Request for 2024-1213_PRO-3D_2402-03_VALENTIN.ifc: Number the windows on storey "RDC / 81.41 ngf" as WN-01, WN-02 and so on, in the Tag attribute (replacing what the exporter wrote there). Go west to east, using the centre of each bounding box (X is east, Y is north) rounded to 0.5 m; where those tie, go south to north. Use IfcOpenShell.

First a look at what the model holds.

```python
import ifcopenshell
import ifcopenshell.util.element
import ifcopenshell.util.placement

model = ifcopenshell.open("2024-1213_PRO-3D_2402-03_VALENTIN.ifc")
print(model.schema)
storey = next(s for s in model.by_type("IfcBuildingStorey") if s.Name == "RDC / 81.41 ngf")
windows = [e for e in ifcopenshell.util.element.get_decomposition(storey) if e.is_a("IfcWindow")]
for e in sorted(windows, key=lambda e: e.id()):
    origin = ifcopenshell.util.placement.get_local_placement(e.ObjectPlacement)[:3, 3]
    print(e.id(), e.Tag, e.Name, origin.round(2) + 0.0, sep=" | ")
```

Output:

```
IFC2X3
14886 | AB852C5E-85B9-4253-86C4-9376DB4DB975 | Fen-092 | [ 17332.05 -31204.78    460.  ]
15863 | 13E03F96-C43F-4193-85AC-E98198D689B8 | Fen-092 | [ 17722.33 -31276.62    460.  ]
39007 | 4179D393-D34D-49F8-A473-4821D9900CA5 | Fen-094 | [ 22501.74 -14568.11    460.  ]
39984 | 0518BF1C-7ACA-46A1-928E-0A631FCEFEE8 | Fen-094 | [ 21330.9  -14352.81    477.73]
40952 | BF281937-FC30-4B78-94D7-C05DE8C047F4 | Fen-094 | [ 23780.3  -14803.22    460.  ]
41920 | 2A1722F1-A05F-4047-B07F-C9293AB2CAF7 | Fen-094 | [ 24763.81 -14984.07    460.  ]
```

```python
import ifcopenshell
import ifcopenshell.geom
import ifcopenshell.util.element
import ifcopenshell.util.shape

model = ifcopenshell.open("2024-1213_PRO-3D_2402-03_VALENTIN.ifc")
settings = ifcopenshell.geom.settings()
settings.set("use-world-coords", True)


def centre(element):
    shape = ifcopenshell.geom.create_shape(settings, element)
    return ifcopenshell.util.shape.get_bbox_centroid(shape.geometry)


storey = next(s for s in model.by_type("IfcBuildingStorey") if s.Name == "RDC / 81.41 ngf")
windows = [e for e in ifcopenshell.util.element.get_decomposition(storey) if e.is_a("IfcWindow")]

# Insertion points can sit at a corner or the storey origin, so sort by the geometry (in metres).
centres = {e: centre(e) for e in windows}
windows.sort(key=lambda e: (round(centres[e][0] / 0.5), centres[e][1]))

for i, e in enumerate(windows, start=1):
    number = f"WN-{i:02d}"
    e.Tag = number
    print(e.id(), number)

model.write("2024-1213_PRO-3D_2402-03_VALENTIN_v2.ifc")
```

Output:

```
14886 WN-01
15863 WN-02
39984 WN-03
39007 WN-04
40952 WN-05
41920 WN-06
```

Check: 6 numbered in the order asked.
